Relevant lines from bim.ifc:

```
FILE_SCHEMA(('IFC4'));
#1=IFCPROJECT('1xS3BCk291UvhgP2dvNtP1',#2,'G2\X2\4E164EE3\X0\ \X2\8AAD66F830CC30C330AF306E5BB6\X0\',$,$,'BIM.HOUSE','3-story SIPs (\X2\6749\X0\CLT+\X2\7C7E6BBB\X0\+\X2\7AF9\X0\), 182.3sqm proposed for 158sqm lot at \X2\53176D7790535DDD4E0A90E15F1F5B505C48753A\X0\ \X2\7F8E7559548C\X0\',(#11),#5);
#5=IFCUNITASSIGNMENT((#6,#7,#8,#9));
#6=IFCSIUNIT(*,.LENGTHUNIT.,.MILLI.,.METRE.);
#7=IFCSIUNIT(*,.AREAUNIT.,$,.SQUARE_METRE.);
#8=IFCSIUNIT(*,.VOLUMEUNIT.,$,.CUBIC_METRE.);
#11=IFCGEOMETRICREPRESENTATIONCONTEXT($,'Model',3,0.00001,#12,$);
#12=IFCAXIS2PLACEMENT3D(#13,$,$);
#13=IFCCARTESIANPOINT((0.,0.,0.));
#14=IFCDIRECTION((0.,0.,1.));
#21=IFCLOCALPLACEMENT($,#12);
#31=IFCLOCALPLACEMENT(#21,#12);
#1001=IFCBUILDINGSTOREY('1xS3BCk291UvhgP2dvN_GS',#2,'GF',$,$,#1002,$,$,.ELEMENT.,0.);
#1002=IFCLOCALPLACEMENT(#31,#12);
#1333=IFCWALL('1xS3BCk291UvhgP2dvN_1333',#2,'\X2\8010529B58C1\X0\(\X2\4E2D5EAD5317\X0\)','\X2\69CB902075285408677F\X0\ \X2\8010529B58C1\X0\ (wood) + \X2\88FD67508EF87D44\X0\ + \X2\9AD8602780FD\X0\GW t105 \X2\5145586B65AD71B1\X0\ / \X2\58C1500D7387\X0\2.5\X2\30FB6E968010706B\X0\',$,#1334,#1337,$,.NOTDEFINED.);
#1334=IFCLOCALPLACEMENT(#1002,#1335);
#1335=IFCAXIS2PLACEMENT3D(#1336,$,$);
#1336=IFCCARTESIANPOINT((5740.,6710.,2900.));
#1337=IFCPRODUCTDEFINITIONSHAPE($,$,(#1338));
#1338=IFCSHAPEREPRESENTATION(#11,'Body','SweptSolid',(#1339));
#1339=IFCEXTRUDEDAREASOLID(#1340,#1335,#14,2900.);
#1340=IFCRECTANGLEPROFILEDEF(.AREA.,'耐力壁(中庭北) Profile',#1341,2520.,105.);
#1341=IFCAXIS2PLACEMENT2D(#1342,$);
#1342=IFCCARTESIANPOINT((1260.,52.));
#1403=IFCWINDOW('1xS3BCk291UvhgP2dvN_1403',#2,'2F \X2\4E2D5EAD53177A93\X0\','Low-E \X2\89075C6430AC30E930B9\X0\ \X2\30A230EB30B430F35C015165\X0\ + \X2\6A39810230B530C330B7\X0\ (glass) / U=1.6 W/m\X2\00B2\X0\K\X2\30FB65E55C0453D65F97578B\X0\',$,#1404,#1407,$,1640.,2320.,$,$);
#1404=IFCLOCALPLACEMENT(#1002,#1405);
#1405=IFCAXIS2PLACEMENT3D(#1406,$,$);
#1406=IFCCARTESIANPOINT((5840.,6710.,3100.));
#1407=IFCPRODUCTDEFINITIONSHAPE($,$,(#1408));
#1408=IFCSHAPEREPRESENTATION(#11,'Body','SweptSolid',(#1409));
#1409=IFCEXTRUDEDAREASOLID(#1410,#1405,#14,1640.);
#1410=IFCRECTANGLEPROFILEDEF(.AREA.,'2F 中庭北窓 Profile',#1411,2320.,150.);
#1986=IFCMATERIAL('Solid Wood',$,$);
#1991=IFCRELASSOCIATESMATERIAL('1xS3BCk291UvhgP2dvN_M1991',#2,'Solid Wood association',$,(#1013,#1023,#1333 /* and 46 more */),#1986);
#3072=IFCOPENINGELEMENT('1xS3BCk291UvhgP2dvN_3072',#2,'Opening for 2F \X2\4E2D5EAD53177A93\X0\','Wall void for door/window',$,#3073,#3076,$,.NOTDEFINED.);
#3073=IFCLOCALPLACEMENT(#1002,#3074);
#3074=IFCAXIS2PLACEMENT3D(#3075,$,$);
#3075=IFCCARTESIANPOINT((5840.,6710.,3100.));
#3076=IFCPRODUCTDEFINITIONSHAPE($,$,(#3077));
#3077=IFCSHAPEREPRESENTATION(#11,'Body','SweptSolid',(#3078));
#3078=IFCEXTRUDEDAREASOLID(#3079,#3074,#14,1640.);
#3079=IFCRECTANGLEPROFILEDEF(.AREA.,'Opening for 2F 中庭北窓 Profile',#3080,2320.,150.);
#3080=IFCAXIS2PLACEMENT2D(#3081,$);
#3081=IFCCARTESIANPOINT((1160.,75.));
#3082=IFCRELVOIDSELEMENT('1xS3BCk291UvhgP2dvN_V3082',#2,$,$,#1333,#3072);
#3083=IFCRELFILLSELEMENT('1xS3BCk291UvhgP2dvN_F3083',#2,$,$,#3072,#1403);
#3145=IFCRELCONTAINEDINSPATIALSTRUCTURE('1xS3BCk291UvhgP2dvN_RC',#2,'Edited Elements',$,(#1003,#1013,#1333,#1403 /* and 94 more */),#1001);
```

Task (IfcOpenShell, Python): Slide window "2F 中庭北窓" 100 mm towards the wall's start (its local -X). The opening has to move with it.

```python
import ifcopenshell
import ifcopenshell.api.geometry
import ifcopenshell.util.placement
import ifcopenshell.util.unit

model = ifcopenshell.open("bim.ifc")
unit_scale = ifcopenshell.util.unit.calculate_unit_scale(model)

window = model.by_guid("1xS3BCk291UvhgP2dvN_1403")
opening = window.FillsVoids[0].RelatingOpeningElement
wall = opening.VoidsElements[0].RelatingBuildingElement

wall_matrix = ifcopenshell.util.placement.get_local_placement(wall.ObjectPlacement)
shift = wall_matrix[:3, 0] * -0.1 / unit_scale
before = ifcopenshell.util.placement.get_local_placement(window.ObjectPlacement)[:3, 3].copy()

# The window is not placed relative to its opening, so move both.
for product in (opening, window):
    matrix = ifcopenshell.util.placement.get_local_placement(product.ObjectPlacement)
    matrix[:3, 3] += shift
    ifcopenshell.api.geometry.edit_object_placement(model, product=product, matrix=matrix, is_si=False)

after = ifcopenshell.util.placement.get_local_placement(window.ObjectPlacement)[:3, 3]
print("window moved by", (after - before).round(3) + 0.0)

model.write("bim_edited.ifc")
```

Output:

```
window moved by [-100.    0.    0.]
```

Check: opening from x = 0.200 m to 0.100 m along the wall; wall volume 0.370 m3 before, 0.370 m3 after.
